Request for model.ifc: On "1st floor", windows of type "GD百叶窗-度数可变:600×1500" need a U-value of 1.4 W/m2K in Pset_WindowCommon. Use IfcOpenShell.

First a look at what the model holds.

```python
import ifcopenshell
import ifcopenshell.util.element

model = ifcopenshell.open("model.ifc")
print(model.schema)
storey = next(s for s in model.by_type("IfcBuildingStorey") if s.Name == "1st floor")
windows = [e for e in ifcopenshell.util.element.get_decomposition(storey) if e.is_a("IfcWindow")]
seen = {}
for e in windows:
    element_type = ifcopenshell.util.element.get_type(e)
    key = (element_type.Name if element_type != e and element_type else None, ifcopenshell.util.element.get_pset(e, "Pset_WindowCommon", "ThermalTransmittance"))
    seen[key] = seen.get(key, 0) + 1
for (name, value), count in sorted(seen.items(), key=str):
    print(count, "x", name, "|", value)
```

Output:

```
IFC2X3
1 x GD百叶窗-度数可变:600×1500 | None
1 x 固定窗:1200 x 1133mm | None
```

```python
import ifcopenshell
import ifcopenshell.api.pset
import ifcopenshell.util.element

model = ifcopenshell.open("model.ifc")

storey = next(s for s in model.by_type("IfcBuildingStorey") if s.Name == "1st floor")
windows = [e for e in ifcopenshell.util.element.get_decomposition(storey) if e.is_a("IfcWindow")]

count = 0
for e in windows:
    element_type = ifcopenshell.util.element.get_type(e)
    if element_type in (None, e) or element_type.Name != "GD百叶窗-度数可变:600×1500":
        continue
    # add_pset returns the element's existing set when there is one.
    pset = ifcopenshell.api.pset.add_pset(model, product=e, name="Pset_WindowCommon")
    ifcopenshell.api.pset.edit_pset(model, pset=pset, properties={"ThermalTransmittance": 1.4})
    count += 1

print(count, "windows updated")

model.write("model_rev.ifc")
```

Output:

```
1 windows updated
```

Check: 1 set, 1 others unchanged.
